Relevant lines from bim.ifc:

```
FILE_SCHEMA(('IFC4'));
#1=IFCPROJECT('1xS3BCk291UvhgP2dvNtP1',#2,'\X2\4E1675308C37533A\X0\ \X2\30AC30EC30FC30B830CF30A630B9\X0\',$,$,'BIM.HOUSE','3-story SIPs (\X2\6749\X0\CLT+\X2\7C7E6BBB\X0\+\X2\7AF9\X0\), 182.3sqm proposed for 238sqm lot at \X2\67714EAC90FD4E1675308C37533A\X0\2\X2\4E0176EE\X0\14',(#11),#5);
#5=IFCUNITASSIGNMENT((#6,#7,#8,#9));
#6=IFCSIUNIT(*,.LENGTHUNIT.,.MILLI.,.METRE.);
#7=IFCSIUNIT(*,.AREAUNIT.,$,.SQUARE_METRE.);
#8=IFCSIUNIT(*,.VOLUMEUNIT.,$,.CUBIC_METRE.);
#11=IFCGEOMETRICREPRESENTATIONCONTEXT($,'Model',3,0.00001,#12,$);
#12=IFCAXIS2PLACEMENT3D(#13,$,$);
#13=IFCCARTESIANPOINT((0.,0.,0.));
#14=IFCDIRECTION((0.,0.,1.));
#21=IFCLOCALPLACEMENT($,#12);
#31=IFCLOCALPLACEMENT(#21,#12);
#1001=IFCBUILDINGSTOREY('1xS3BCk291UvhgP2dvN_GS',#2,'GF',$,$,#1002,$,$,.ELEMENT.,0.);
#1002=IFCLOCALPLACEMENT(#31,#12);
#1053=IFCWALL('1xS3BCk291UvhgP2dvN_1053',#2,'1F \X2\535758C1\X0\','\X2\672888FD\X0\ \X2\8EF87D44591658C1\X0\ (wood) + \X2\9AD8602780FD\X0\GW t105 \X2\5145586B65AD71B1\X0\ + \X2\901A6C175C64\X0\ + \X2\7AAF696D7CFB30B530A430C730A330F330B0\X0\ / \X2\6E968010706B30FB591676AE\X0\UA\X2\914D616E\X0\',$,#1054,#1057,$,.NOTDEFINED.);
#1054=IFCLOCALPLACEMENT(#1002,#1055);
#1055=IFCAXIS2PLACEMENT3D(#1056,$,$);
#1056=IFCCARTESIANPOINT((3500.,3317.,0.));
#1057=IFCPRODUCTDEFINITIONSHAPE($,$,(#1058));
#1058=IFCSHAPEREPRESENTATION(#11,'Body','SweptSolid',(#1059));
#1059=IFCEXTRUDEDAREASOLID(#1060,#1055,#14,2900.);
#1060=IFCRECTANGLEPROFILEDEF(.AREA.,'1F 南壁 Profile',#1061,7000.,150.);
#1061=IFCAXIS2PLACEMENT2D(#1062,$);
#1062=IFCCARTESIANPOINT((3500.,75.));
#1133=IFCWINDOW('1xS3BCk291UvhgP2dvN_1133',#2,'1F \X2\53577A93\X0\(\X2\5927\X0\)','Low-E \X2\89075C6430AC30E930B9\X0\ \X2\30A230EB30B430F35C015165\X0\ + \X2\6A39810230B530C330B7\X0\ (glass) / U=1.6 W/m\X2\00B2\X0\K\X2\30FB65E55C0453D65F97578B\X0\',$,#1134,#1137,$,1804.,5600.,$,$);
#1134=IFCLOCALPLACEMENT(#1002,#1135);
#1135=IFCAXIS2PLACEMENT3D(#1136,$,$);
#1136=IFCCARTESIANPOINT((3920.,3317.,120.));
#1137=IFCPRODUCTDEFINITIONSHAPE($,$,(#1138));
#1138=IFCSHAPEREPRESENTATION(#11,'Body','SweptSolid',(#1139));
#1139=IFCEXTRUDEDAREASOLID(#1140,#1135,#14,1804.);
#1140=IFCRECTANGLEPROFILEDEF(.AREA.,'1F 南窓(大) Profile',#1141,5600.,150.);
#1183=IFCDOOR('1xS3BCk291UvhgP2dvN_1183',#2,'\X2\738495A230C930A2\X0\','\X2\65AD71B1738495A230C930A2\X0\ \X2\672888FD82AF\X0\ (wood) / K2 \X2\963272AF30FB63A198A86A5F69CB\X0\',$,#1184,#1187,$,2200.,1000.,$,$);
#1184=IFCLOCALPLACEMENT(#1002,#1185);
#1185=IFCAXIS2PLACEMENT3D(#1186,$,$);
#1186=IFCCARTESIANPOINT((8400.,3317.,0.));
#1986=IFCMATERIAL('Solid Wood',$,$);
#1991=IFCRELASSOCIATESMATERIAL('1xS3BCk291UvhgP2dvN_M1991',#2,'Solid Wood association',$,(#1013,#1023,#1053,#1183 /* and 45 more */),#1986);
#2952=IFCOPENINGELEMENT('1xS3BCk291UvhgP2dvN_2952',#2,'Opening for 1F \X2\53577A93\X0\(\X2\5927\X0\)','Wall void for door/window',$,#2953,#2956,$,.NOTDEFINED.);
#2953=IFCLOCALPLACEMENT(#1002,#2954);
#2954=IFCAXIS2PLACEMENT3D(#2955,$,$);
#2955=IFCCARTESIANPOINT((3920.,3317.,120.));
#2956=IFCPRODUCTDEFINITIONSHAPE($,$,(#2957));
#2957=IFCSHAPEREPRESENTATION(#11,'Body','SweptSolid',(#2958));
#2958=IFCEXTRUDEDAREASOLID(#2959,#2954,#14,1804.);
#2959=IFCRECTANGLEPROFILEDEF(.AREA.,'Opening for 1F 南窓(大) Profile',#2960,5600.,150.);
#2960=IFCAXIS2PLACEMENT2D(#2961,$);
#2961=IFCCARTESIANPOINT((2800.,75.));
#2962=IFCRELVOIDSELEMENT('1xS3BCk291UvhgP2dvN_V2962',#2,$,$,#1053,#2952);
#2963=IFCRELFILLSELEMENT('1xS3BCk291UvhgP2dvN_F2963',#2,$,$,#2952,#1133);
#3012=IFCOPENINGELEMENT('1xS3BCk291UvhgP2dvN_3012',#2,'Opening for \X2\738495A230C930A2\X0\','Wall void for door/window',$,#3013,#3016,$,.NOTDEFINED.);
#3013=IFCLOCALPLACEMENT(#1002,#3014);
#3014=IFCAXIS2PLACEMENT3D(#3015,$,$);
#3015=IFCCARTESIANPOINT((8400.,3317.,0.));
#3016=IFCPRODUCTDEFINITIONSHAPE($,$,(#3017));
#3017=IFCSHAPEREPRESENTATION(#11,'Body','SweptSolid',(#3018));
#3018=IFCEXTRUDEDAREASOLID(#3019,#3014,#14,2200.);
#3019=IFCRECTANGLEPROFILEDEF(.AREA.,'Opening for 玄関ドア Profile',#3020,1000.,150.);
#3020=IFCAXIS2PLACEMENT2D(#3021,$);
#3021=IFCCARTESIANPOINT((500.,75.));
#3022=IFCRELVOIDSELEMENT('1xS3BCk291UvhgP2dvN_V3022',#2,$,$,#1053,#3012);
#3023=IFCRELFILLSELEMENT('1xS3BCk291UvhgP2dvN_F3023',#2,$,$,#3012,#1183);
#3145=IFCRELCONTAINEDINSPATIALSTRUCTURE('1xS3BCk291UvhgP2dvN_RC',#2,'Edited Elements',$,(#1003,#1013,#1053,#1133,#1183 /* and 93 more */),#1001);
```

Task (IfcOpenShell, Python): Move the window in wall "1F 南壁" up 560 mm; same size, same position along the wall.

```python
import numpy as np
import ifcopenshell
import ifcopenshell.api.geometry
import ifcopenshell.util.placement
import ifcopenshell.util.unit

model = ifcopenshell.open("bim.ifc")
unit_scale = ifcopenshell.util.unit.calculate_unit_scale(model)

window = model.by_guid("1xS3BCk291UvhgP2dvN_1133")
opening = window.FillsVoids[0].RelatingOpeningElement
dz = 0.56 / unit_scale

shift = np.array([0.0, 0.0, dz])
# The window is not placed relative to its opening, so move both.
for product in (opening, window):
    matrix = ifcopenshell.util.placement.get_local_placement(product.ObjectPlacement)
    matrix[:3, 3] += shift
    ifcopenshell.api.geometry.edit_object_placement(model, product=product, matrix=matrix, is_si=False)

print(f"moved by {dz * unit_scale:+.3f} m")

model.write("bim-out.ifc")
```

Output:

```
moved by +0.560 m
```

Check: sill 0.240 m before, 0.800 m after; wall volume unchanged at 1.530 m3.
